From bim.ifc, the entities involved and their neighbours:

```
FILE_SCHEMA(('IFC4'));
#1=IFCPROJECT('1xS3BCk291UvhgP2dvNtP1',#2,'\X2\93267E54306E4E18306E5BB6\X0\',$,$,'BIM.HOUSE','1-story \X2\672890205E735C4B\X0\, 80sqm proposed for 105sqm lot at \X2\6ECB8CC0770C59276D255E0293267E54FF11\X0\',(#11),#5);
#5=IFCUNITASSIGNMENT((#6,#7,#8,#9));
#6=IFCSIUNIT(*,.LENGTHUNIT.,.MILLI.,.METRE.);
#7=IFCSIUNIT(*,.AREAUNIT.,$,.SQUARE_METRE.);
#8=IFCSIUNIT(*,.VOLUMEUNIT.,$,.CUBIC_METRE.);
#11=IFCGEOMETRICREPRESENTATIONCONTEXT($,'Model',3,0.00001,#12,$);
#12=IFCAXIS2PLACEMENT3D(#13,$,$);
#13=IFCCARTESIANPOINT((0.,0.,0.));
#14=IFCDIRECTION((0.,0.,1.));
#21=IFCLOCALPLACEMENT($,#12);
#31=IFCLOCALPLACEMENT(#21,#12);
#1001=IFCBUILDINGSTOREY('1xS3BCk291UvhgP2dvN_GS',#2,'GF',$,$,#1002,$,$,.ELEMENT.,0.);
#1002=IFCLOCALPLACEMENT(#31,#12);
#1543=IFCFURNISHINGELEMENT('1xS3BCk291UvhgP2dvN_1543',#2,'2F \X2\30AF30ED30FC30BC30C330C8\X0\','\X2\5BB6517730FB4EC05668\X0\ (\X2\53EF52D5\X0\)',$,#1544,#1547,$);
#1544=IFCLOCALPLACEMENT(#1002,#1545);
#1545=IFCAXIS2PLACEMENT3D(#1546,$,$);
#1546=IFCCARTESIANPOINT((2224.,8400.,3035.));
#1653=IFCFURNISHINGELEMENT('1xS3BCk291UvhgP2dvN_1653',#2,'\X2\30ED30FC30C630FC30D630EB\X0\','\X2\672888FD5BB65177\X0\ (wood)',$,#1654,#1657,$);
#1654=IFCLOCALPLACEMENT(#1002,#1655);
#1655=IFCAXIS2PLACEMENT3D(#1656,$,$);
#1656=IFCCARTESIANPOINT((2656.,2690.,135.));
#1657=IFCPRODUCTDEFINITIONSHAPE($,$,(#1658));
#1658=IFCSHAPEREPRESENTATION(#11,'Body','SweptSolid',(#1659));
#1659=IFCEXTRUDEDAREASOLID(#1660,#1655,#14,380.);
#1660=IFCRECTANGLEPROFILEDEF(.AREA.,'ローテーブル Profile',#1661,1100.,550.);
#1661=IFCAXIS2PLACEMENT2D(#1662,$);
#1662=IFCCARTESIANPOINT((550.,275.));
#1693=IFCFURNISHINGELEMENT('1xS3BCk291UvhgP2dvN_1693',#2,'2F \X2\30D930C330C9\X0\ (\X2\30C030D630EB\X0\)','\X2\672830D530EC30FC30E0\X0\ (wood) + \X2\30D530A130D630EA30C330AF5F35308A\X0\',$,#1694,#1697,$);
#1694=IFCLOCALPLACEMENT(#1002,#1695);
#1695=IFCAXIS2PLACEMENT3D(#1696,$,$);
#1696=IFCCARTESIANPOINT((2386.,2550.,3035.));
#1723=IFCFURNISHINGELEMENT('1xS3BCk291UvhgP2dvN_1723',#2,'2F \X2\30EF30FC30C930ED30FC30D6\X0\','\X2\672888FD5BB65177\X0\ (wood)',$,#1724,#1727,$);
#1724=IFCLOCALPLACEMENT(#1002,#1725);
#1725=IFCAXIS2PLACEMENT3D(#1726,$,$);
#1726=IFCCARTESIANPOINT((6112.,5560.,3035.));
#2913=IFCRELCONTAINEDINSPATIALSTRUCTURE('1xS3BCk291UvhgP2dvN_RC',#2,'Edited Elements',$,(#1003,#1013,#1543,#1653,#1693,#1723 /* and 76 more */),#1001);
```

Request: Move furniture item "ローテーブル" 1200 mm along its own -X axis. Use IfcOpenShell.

```python
import ifcopenshell
import ifcopenshell.api.geometry
import ifcopenshell.util.placement
import ifcopenshell.util.unit

model = ifcopenshell.open("bim.ifc")
unit_scale = ifcopenshell.util.unit.calculate_unit_scale(model)

item = model.by_guid("1xS3BCk291UvhgP2dvN_1653")
matrix = ifcopenshell.util.placement.get_local_placement(item.ObjectPlacement)
matrix[:3, 3] -= matrix[:3, 0] * 1.2 / unit_scale
ifcopenshell.api.geometry.edit_object_placement(model, product=item, matrix=matrix, is_si=False)

print(ifcopenshell.util.placement.get_local_placement(item.ObjectPlacement).round(3) + 0.0)

model.write("bim_edited.ifc")
```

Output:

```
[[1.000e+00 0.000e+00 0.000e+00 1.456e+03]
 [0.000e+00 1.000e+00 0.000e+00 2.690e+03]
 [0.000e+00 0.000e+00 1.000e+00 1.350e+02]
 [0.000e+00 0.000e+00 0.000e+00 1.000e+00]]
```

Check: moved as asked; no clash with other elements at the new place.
